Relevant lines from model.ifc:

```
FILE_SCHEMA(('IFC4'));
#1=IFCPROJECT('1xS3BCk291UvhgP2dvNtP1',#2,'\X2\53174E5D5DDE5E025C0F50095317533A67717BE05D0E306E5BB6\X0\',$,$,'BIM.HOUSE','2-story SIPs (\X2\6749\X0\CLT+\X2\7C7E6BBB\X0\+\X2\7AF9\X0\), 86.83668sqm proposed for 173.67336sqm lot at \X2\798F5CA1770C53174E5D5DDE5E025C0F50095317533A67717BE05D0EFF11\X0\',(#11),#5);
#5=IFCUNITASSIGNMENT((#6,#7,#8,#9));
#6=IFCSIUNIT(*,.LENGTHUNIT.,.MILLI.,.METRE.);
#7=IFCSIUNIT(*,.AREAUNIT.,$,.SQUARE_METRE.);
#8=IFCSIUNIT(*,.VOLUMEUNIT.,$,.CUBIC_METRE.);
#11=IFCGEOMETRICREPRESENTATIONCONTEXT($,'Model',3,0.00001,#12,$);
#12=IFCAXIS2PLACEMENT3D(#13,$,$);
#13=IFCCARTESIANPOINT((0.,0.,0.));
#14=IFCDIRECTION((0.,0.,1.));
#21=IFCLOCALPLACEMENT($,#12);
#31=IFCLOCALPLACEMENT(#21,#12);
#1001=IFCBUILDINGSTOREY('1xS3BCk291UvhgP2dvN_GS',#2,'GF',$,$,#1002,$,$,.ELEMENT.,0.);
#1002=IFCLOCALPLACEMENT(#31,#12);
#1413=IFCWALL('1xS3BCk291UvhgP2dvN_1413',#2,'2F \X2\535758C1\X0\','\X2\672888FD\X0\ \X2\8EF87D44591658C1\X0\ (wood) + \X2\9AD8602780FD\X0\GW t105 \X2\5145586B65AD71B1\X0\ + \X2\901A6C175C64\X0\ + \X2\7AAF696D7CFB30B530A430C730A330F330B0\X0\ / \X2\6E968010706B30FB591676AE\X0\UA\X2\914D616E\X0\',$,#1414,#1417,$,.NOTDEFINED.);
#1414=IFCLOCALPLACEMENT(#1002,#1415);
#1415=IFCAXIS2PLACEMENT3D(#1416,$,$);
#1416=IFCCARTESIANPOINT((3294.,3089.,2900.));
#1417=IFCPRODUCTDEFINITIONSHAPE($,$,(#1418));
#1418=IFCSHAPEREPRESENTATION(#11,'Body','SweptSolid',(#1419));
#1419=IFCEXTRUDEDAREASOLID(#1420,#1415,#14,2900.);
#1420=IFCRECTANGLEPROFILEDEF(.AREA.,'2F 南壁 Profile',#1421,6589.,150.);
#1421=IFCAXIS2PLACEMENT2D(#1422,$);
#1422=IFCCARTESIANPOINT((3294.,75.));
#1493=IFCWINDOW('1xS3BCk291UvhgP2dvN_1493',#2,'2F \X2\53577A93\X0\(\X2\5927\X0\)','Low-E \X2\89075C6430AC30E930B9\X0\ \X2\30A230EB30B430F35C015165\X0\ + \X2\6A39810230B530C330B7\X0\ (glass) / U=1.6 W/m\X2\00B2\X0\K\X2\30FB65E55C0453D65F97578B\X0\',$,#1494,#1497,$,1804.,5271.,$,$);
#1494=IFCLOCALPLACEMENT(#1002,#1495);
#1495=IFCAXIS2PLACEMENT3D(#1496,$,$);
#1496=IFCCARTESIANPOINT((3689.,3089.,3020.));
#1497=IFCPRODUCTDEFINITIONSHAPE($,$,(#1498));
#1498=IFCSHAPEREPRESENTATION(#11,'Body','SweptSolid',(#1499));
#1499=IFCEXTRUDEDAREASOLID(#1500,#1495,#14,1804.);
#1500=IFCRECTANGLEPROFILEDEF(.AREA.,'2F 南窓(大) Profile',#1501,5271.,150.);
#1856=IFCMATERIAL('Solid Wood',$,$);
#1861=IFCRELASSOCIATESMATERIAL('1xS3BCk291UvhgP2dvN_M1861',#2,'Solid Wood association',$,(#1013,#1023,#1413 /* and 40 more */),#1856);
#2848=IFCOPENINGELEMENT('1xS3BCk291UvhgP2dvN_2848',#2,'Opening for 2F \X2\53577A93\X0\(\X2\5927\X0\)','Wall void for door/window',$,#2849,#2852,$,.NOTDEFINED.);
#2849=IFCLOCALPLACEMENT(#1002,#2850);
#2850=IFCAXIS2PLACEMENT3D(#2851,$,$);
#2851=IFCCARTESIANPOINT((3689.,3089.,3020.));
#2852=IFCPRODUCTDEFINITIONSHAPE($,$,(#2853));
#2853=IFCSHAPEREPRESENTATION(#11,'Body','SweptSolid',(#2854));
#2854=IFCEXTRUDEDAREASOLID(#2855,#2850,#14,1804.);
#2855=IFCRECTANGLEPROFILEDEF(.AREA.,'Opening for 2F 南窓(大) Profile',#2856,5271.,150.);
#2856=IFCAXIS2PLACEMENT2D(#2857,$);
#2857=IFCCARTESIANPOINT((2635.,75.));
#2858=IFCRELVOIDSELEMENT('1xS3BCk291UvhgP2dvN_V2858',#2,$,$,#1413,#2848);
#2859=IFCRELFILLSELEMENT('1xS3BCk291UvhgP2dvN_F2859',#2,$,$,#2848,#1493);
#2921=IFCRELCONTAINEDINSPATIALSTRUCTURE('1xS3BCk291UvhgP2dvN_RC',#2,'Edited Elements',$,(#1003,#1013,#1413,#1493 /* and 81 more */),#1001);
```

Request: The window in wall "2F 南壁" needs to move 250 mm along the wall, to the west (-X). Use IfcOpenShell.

```python
import ifcopenshell
import ifcopenshell.api.geometry
import ifcopenshell.util.placement

model = ifcopenshell.open("model.ifc")

window = model.by_guid("1xS3BCk291UvhgP2dvN_1493")
opening = window.FillsVoids[0].RelatingOpeningElement
wall = opening.VoidsElements[0].RelatingBuildingElement

wall_matrix = ifcopenshell.util.placement.get_local_placement(wall.ObjectPlacement)
shift = wall_matrix[:3, 0] * -250.0
before = ifcopenshell.util.placement.get_local_placement(window.ObjectPlacement)[:3, 3].copy()

# The window is not placed relative to its opening, so move both.
for product in (opening, window):
    matrix = ifcopenshell.util.placement.get_local_placement(product.ObjectPlacement)
    matrix[:3, 3] += shift
    ifcopenshell.api.geometry.edit_object_placement(model, product=product, matrix=matrix, is_si=False)

after = ifcopenshell.util.placement.get_local_placement(window.ObjectPlacement)[:3, 3]
print("window moved by", (after - before).round(3) + 0.0)

model.write("model_updated.ifc")
```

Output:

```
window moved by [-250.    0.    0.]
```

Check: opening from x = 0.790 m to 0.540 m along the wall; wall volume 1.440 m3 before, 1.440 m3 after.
